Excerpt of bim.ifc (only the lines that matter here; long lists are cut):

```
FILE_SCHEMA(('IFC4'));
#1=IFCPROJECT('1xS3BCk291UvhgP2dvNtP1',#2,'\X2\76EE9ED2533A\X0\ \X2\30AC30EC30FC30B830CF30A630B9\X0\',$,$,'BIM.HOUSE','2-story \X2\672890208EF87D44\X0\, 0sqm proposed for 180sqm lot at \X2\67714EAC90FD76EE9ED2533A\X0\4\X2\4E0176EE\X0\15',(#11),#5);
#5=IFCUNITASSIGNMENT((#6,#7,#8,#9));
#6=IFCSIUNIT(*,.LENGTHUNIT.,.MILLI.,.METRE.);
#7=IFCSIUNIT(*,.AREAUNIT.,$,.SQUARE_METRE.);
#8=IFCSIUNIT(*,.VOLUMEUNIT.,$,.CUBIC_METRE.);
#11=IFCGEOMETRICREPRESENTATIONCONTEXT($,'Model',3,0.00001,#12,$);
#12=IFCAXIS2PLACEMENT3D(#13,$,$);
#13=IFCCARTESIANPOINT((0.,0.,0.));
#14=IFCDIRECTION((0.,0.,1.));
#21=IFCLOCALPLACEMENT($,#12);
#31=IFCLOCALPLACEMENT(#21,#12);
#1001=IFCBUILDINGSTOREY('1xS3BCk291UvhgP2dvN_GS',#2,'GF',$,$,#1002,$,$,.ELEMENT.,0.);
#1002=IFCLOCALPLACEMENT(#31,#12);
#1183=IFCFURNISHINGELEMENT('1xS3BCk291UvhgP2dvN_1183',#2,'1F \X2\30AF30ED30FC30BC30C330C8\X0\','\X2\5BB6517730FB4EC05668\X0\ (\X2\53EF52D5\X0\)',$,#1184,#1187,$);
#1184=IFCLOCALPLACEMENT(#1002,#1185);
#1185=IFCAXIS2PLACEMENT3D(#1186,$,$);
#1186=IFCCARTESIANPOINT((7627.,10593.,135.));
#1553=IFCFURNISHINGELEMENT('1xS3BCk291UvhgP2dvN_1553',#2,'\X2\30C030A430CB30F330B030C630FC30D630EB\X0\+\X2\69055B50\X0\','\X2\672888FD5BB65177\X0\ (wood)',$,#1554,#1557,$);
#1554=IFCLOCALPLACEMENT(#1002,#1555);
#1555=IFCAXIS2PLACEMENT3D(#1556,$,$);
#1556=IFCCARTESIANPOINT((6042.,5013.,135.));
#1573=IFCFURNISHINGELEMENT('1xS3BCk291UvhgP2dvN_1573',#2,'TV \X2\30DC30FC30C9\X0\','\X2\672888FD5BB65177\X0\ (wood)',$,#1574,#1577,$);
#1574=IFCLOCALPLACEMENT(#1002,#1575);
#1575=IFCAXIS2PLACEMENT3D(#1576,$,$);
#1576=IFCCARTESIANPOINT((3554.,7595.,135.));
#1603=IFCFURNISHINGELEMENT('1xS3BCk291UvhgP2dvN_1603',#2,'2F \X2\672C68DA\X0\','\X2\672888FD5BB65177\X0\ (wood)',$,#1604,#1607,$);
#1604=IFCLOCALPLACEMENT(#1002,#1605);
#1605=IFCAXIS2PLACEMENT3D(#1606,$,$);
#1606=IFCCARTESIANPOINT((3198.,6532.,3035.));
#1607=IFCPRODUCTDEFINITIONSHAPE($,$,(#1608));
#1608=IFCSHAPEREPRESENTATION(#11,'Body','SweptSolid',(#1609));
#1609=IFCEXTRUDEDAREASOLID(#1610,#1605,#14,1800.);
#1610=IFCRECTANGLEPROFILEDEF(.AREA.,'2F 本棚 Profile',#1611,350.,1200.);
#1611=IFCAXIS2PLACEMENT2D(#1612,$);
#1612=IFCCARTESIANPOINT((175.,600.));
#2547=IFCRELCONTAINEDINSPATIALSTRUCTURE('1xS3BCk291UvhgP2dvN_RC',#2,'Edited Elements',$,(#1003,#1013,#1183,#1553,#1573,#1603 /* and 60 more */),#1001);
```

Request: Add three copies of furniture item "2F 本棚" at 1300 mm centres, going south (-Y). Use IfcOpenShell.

```python
import numpy as np
import ifcopenshell
import ifcopenshell.api.geometry
import ifcopenshell.api.root
import ifcopenshell.util.element
import ifcopenshell.util.placement
import ifcopenshell.util.unit

model = ifcopenshell.open("bim.ifc")
unit_scale = ifcopenshell.util.unit.calculate_unit_scale(model)


def reuse_history(source, copy):
    """copy_class also copies each property set's owner history, people and application; keep the originals."""
    for rel in copy.IsDefinedBy:
        if rel.is_a("IfcRelDefinesByProperties") and (history := rel.RelatingPropertyDefinition.OwnerHistory):
            rel.RelatingPropertyDefinition.OwnerHistory = source.OwnerHistory
            ifcopenshell.util.element.remove_deep2(model, history)


source = model.by_guid("1xS3BCk291UvhgP2dvN_1603")
base = ifcopenshell.util.placement.get_local_placement(source.ObjectPlacement)
step = np.array([0.0, -1.0, 0.0]) * 1.3 / unit_scale

for i in range(1, 4):
    copy = ifcopenshell.api.root.copy_class(model, product=source)
    copy.Representation = ifcopenshell.util.element.copy_deep(
        model, source.Representation, exclude=["IfcGeometricRepresentationContext", "IfcRepresentationMap"]
    )
    reuse_history(source, copy)
    matrix = base.copy()
    matrix[:3, 3] += i * step
    print("added at", matrix[:3, 3].round(3) + 0.0)
    ifcopenshell.api.geometry.edit_object_placement(model, product=copy, matrix=matrix, is_si=False)

model.write("bim_updated.ifc")
```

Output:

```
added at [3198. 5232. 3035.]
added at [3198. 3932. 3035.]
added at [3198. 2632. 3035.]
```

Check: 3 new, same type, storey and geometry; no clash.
